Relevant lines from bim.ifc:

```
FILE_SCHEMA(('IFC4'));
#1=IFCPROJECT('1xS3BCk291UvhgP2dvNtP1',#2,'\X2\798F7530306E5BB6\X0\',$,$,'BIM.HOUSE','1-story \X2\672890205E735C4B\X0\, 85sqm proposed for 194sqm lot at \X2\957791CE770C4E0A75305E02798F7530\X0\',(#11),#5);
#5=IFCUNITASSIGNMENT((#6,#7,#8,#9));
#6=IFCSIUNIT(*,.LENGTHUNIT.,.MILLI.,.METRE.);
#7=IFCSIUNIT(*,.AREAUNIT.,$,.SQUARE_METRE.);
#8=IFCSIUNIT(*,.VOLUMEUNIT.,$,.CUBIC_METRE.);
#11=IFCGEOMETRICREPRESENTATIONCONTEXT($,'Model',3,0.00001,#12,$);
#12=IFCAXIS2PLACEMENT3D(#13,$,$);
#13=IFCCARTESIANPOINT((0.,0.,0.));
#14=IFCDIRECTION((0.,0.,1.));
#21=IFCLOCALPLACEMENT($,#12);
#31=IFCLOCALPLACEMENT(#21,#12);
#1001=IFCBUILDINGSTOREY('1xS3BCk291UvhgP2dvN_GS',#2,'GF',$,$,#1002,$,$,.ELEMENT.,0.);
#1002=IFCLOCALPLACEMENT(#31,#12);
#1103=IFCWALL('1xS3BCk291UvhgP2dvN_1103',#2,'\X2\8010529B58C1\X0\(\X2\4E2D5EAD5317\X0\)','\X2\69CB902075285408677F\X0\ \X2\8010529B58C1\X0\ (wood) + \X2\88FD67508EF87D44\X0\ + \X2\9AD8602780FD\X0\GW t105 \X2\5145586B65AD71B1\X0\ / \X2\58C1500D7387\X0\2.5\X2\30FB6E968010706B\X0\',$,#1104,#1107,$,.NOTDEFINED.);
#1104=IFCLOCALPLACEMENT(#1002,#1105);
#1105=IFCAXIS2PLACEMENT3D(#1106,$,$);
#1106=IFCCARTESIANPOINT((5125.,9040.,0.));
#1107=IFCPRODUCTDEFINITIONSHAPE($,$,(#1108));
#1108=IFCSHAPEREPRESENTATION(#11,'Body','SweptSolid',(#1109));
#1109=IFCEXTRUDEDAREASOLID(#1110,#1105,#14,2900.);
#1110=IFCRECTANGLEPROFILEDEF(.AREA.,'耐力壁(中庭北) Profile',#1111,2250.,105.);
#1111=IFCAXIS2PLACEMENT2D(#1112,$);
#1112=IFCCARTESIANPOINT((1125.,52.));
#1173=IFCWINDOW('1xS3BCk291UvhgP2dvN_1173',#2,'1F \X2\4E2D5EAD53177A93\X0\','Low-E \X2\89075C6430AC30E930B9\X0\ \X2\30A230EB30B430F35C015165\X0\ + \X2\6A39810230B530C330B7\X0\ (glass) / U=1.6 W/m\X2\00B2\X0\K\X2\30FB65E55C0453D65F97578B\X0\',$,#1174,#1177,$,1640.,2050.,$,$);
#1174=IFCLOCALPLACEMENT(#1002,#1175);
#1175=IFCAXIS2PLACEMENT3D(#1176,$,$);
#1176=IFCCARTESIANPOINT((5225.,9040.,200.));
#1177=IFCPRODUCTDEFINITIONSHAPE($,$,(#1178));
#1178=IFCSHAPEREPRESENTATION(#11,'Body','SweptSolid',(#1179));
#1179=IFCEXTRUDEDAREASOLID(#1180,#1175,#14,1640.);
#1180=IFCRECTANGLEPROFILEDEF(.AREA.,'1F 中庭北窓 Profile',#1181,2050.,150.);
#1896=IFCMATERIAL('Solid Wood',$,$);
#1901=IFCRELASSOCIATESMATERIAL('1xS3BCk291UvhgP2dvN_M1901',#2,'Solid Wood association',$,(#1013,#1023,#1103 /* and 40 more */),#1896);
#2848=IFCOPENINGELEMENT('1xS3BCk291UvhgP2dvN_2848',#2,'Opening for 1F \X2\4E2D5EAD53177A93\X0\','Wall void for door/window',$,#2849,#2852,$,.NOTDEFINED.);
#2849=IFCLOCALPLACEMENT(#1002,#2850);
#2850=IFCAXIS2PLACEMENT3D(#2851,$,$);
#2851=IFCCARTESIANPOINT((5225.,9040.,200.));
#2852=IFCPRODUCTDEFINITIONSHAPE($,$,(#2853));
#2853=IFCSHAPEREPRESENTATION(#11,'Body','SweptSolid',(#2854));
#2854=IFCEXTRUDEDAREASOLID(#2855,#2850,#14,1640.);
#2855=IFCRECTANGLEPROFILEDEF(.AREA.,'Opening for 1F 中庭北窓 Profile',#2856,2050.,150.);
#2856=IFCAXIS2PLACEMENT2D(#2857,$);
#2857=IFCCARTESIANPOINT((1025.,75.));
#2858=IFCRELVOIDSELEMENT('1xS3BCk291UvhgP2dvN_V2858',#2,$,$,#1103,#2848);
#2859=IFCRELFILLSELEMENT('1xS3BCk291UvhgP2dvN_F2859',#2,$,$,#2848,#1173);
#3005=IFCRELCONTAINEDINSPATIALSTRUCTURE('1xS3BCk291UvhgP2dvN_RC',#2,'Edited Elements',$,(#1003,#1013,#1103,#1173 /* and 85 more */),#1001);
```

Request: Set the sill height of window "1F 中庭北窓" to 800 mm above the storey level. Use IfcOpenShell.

```python
import numpy as np
import ifcopenshell
import ifcopenshell.api.geometry
import ifcopenshell.geom
import ifcopenshell.util.element
import ifcopenshell.util.placement
import ifcopenshell.util.shape
import ifcopenshell.util.unit

model = ifcopenshell.open("bim.ifc")
unit_scale = ifcopenshell.util.unit.calculate_unit_scale(model)

window = model.by_guid("1xS3BCk291UvhgP2dvN_1173")
opening = window.FillsVoids[0].RelatingOpeningElement
storey = ifcopenshell.util.element.get_container(window, ifc_class="IfcBuildingStorey")
level = ifcopenshell.util.placement.get_local_placement(storey.ObjectPlacement)[2, 3]

# The opening's origin need not be at the sill, so measure its lowest point.
shape = ifcopenshell.geom.create_shape(ifcopenshell.geom.settings(), opening)
bottom = ifcopenshell.util.shape.get_shape_bottom_elevation(shape, shape.geometry) / unit_scale
dz = level + 800.0 - bottom

shift = np.array([0.0, 0.0, dz])
# The window is not placed relative to its opening, so move both.
for product in (opening, window):
    matrix = ifcopenshell.util.placement.get_local_placement(product.ObjectPlacement)
    matrix[:3, 3] += shift
    ifcopenshell.api.geometry.edit_object_placement(model, product=product, matrix=matrix, is_si=False)

print(f"moved by {dz * unit_scale:+.3f} m")

model.write("bim_v2.ifc")
```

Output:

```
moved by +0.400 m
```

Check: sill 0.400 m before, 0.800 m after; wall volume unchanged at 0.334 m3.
